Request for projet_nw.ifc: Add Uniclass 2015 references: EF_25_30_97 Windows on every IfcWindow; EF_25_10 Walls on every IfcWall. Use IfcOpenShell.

First a look at what the model holds.

```python
import ifcopenshell

model = ifcopenshell.open("projet_nw.ifc")
print(model.schema)
print("classifications:", [c.Name for c in model.by_type("IfcClassification")])
for ifc_class in ("IfcDoor", "IfcRoof", "IfcStair", "IfcWall", "IfcWindow"):
    print(ifc_class, len(model.by_type(ifc_class)))
```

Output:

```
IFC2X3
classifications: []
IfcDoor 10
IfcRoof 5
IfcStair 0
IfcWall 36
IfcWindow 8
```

```python
import ifcopenshell
import ifcopenshell.api.classification

model = ifcopenshell.open("projet_nw.ifc")

# IFC2X3 requires Source and Edition and has no link from the project to the system.
system = model.create_entity("IfcClassification", Source="NBS", Edition="2015", Name="Uniclass 2015")

codes = {
    "IfcWindow": ("EF_25_30_97", "Windows"),
    "IfcWall": ("EF_25_10", "Walls"),
}
for ifc_class, (code, name) in codes.items():
    products = model.by_type(ifc_class)
    ifcopenshell.api.classification.add_reference(
        model, products=products, classification=system, identification=code, name=name
    )
    print(code, len(products))

model.write("projet_nw_v2.ifc")
```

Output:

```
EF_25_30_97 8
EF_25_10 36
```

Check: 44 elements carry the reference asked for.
